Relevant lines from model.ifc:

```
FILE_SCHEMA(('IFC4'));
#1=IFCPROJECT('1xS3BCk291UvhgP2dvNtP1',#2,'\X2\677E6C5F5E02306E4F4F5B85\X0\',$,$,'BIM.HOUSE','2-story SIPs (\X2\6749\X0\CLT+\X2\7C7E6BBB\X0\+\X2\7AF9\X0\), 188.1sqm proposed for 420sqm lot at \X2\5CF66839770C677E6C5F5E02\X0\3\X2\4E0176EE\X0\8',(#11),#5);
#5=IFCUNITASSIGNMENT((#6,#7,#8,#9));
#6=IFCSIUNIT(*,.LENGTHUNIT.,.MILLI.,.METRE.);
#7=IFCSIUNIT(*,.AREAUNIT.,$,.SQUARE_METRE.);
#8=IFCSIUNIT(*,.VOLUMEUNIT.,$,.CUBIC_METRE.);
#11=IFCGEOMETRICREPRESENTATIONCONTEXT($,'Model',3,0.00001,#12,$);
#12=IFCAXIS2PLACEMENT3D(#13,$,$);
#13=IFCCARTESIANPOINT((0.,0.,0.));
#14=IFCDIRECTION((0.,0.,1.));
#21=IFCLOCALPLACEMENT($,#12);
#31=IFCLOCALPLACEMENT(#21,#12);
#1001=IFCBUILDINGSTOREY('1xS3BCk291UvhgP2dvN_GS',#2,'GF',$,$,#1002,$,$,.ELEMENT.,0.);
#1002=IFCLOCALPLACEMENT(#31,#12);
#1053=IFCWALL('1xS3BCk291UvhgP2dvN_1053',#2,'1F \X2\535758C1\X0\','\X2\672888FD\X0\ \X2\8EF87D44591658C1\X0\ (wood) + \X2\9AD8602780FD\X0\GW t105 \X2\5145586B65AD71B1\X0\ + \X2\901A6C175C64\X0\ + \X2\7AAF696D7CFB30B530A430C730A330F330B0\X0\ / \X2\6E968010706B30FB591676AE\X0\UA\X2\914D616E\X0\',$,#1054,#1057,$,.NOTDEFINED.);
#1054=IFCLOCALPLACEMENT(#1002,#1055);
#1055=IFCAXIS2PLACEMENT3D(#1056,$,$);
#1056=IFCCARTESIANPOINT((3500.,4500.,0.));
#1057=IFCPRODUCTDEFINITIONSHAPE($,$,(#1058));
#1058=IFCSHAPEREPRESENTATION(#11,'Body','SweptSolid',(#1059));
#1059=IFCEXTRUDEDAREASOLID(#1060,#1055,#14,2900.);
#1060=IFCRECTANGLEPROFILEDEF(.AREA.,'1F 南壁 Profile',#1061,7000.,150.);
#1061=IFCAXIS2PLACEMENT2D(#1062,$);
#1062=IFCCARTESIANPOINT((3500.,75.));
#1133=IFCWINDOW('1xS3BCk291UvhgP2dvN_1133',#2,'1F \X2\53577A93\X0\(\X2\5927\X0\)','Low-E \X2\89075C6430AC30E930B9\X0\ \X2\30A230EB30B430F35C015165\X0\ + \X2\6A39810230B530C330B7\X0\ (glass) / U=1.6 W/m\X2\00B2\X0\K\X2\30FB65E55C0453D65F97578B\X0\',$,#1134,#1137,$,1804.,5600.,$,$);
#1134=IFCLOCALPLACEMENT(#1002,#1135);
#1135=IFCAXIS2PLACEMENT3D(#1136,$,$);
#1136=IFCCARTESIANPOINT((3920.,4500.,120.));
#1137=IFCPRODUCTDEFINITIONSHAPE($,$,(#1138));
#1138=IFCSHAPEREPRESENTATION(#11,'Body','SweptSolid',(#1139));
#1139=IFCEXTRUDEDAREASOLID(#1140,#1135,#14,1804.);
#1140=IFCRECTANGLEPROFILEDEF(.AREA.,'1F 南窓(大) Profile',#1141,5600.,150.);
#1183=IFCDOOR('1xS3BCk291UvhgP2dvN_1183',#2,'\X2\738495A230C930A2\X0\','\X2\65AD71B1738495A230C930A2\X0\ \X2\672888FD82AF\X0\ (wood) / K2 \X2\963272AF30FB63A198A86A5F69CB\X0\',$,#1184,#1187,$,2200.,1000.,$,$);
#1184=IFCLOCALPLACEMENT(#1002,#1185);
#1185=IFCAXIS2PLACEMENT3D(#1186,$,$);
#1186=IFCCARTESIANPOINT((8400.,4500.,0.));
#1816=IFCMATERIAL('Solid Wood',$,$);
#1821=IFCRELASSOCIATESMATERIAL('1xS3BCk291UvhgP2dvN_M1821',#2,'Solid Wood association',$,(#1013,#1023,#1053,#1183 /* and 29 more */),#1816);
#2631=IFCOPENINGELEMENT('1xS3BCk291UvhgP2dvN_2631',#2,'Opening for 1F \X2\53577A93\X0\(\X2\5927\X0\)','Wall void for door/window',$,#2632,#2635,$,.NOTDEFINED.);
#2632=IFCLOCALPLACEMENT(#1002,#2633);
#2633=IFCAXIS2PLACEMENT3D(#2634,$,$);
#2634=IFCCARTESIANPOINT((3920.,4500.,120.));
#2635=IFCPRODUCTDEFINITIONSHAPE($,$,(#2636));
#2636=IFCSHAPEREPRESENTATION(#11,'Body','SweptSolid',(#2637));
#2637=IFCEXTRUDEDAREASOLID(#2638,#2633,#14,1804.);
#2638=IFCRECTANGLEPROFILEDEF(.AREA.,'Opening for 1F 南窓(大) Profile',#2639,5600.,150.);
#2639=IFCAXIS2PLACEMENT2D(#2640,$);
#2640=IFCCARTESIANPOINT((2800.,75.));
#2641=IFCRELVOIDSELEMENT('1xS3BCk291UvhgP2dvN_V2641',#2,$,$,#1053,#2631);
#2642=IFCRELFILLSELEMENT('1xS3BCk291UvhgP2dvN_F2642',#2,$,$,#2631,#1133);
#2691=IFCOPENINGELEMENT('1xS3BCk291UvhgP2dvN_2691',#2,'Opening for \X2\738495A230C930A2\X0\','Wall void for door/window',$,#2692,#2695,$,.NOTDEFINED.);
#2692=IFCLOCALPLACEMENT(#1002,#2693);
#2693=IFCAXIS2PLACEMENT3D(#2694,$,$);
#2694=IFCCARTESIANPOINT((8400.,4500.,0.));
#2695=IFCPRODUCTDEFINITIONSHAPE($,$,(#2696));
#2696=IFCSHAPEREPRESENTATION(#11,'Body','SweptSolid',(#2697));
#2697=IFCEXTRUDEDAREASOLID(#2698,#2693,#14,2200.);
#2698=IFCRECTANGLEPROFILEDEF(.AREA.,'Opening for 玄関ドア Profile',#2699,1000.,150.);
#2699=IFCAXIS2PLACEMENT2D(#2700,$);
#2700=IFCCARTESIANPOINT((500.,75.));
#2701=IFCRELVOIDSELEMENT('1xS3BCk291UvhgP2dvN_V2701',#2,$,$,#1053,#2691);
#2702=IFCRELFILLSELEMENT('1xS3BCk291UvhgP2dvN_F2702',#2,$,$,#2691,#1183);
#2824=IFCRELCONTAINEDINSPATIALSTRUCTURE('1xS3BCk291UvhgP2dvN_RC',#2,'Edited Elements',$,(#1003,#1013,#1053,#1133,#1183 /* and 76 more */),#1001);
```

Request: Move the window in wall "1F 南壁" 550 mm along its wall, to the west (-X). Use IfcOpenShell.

```python
import ifcopenshell
import ifcopenshell.api.geometry
import ifcopenshell.util.placement

model = ifcopenshell.open("model.ifc")

window = model.by_guid("1xS3BCk291UvhgP2dvN_1133")
opening = window.FillsVoids[0].RelatingOpeningElement
wall = opening.VoidsElements[0].RelatingBuildingElement

wall_matrix = ifcopenshell.util.placement.get_local_placement(wall.ObjectPlacement)
shift = wall_matrix[:3, 0] * -550.0
before = ifcopenshell.util.placement.get_local_placement(window.ObjectPlacement)[:3, 3].copy()

# The window is not placed relative to its opening, so move both.
for product in (opening, window):
    matrix = ifcopenshell.util.placement.get_local_placement(product.ObjectPlacement)
    matrix[:3, 3] += shift
    ifcopenshell.api.geometry.edit_object_placement(model, product=product, matrix=matrix, is_si=False)

after = ifcopenshell.util.placement.get_local_placement(window.ObjectPlacement)[:3, 3]
print("window moved by", (after - before).round(3) + 0.0)

model.write("model_updated.ifc")
```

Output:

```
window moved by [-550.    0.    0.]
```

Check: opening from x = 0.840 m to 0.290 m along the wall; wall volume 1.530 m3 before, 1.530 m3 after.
